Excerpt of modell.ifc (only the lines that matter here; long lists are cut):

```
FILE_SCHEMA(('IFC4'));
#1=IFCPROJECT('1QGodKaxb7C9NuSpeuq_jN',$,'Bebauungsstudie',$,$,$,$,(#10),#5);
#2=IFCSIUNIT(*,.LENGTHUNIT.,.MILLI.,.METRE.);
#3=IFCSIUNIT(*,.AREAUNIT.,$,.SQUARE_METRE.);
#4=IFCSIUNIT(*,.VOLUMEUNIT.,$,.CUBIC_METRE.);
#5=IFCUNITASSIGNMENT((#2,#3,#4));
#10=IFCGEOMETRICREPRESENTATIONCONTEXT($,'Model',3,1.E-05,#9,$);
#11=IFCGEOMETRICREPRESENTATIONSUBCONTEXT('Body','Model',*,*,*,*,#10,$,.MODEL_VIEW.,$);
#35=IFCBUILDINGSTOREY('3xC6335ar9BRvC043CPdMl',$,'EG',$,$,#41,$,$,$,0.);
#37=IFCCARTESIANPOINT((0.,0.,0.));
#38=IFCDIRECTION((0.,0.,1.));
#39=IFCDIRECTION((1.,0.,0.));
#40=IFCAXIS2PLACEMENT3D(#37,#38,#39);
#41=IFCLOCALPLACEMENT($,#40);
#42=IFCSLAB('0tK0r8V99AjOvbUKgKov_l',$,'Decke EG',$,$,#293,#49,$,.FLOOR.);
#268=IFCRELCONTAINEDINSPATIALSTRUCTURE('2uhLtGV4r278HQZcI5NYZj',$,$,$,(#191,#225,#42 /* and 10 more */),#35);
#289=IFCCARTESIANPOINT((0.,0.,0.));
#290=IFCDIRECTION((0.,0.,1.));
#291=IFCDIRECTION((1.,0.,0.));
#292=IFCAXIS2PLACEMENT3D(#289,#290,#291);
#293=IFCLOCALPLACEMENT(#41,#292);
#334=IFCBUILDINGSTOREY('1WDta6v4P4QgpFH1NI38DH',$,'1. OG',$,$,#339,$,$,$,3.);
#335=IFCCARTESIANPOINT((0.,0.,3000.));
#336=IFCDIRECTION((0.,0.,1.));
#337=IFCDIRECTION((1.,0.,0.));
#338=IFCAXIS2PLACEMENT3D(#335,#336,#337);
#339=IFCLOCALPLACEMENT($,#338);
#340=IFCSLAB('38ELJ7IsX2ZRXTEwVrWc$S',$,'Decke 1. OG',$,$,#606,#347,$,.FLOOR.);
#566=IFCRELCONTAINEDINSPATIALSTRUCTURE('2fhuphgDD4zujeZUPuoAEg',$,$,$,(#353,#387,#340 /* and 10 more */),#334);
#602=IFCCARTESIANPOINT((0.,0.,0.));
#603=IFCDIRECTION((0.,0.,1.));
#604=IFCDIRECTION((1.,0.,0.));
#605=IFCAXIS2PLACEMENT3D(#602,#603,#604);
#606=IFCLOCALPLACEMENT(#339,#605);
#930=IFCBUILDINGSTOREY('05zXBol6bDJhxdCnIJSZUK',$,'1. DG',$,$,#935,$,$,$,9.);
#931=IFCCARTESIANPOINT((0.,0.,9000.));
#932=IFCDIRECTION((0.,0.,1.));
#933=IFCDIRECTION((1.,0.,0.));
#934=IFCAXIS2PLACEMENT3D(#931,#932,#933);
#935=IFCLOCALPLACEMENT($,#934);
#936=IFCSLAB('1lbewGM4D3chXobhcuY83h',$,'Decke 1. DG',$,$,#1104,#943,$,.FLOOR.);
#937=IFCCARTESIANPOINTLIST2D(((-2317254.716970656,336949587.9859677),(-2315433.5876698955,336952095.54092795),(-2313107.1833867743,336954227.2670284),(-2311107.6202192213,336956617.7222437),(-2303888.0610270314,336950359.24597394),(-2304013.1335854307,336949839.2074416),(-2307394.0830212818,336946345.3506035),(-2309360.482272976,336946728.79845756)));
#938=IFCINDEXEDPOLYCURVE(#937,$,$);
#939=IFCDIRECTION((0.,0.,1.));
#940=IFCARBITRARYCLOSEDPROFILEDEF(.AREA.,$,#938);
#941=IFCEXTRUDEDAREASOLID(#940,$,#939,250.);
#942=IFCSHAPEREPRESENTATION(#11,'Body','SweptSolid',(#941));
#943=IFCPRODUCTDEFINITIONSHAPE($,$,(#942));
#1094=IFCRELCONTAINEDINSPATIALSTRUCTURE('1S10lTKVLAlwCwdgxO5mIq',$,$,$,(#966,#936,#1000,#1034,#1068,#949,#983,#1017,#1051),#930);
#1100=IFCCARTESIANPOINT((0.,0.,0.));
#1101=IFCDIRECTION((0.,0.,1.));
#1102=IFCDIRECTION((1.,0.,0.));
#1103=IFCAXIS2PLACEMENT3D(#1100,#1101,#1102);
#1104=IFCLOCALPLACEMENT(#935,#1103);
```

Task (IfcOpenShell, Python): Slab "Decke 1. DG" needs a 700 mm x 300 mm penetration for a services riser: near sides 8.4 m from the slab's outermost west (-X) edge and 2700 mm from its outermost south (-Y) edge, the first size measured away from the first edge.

```python
import numpy as np
import ifcopenshell
import ifcopenshell.api.feature
import ifcopenshell.api.geometry
import ifcopenshell.api.root
import ifcopenshell.geom
import ifcopenshell.util.placement
import ifcopenshell.util.representation
import ifcopenshell.util.shape
import ifcopenshell.util.unit

model = ifcopenshell.open("modell.ifc")
unit_scale = ifcopenshell.util.unit.calculate_unit_scale(model)
settings = ifcopenshell.geom.settings()


def volume(element):
    """Net volume in cubic metres, openings subtracted."""
    shape = ifcopenshell.geom.create_shape(settings, element)
    return ifcopenshell.util.shape.get_volume(shape.geometry)


slab = model.by_guid("1lbewGM4D3chXobhcuY83h")
before = volume(slab)

# Extent in the slab's own axes, in metres. The edges named are its -X and -Y sides.
slab_shape = ifcopenshell.geom.create_shape(settings, slab)
vertices = ifcopenshell.util.shape.get_vertices(slab_shape.geometry)
x_min, y_min, bottom = vertices.min(axis=0)
top = vertices[:, 2].max()

opening = ifcopenshell.api.root.create_entity(model, ifc_class="IfcOpeningElement", name="Services riser opening", predefined_type="OPENING")
context = ifcopenshell.util.representation.get_context(model, "Model", "Body", "MODEL_VIEW")
width, depth = 0.7, 0.3
outline = [(0.0, 0.0), (width, 0.0), (width, depth), (0.0, depth), (0.0, 0.0)]
# Overshoot both faces by 50 mm so the cut is clean.
shape = ifcopenshell.api.geometry.add_slab_representation(
    model, context=context, depth=top - bottom + 0.1, polyline=outline
)
ifcopenshell.api.geometry.assign_representation(model, product=opening, representation=shape)

matrix = ifcopenshell.util.placement.get_local_placement(slab.ObjectPlacement)
matrix[:, 3] = matrix @ np.append(np.array([x_min + 8.4, y_min + 2.7, bottom - 0.05]) / unit_scale, 1.0)
ifcopenshell.api.geometry.edit_object_placement(model, product=opening, matrix=matrix, is_si=False)
ifcopenshell.api.feature.add_feature(model, feature=opening, element=slab)

after = volume(slab)

print(f"slab volume {before:.3f} -> {after:.3f} m3")

model.write("modell-out.ifc")
```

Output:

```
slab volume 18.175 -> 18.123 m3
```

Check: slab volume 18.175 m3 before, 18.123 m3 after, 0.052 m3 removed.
